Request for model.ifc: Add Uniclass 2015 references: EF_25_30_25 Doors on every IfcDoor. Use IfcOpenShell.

First a look at what the model holds.

```python
import ifcopenshell

model = ifcopenshell.open("model.ifc")
print(model.schema)
print("classifications:", [c.Name for c in model.by_type("IfcClassification")])
for ifc_class in ("IfcDoor", "IfcRoof", "IfcStair", "IfcWall", "IfcWindow"):
    print(ifc_class, len(model.by_type(ifc_class)))
```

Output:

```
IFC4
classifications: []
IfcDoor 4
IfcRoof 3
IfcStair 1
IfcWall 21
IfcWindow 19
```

```python
import ifcopenshell
import ifcopenshell.api.classification

model = ifcopenshell.open("model.ifc")

system = ifcopenshell.api.classification.add_classification(model, classification="Uniclass 2015")

codes = {
    "IfcDoor": ("EF_25_30_25", "Doors"),
}
for ifc_class, (code, name) in codes.items():
    products = model.by_type(ifc_class)
    ifcopenshell.api.classification.add_reference(
        model, products=products, classification=system, identification=code, name=name
    )
    print(code, len(products))

model.write("model_rev.ifc")
```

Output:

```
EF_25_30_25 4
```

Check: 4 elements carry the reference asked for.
